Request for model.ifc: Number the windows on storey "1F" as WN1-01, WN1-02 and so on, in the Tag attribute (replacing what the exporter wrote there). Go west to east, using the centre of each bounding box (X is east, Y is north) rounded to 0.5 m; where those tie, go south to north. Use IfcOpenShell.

First a look at what the model holds.

```python
import ifcopenshell
import ifcopenshell.util.element
import ifcopenshell.util.placement

model = ifcopenshell.open("model.ifc")
print(model.schema)
storey = next(s for s in model.by_type("IfcBuildingStorey") if s.Name == "1F")
windows = [e for e in ifcopenshell.util.element.get_decomposition(storey) if e.is_a("IfcWindow")]
for e in sorted(windows, key=lambda e: e.id()):
    origin = ifcopenshell.util.placement.get_local_placement(e.ObjectPlacement)[:3, 3]
    print(e.id(), e.Tag, e.Name, origin.round(2) + 0.0, sep=" | ")
```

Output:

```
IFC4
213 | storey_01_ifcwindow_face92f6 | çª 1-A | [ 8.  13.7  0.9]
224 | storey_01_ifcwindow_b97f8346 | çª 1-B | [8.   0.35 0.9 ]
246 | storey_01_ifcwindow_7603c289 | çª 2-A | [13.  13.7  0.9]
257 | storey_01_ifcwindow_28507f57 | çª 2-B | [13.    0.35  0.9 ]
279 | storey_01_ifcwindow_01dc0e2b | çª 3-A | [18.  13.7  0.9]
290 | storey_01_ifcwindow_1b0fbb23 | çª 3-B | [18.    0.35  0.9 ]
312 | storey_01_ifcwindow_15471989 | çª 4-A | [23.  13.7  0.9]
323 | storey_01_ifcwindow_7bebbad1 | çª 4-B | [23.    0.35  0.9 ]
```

```python
import ifcopenshell
import ifcopenshell.geom
import ifcopenshell.util.element
import ifcopenshell.util.shape

model = ifcopenshell.open("model.ifc")
settings = ifcopenshell.geom.settings()
settings.set("use-world-coords", True)


def centre(element):
    shape = ifcopenshell.geom.create_shape(settings, element)
    return ifcopenshell.util.shape.get_bbox_centroid(shape.geometry)


storey = next(s for s in model.by_type("IfcBuildingStorey") if s.Name == "1F")
windows = [e for e in ifcopenshell.util.element.get_decomposition(storey) if e.is_a("IfcWindow")]

# Insertion points can sit at a corner or the storey origin, so sort by the geometry (in metres).
centres = {e: centre(e) for e in windows}
windows.sort(key=lambda e: (round(centres[e][0] / 0.5), centres[e][1]))

for i, e in enumerate(windows, start=1):
    number = f"WN1-{i:02d}"
    e.Tag = number
    print(e.id(), number)

model.write("model_edited.ifc")
```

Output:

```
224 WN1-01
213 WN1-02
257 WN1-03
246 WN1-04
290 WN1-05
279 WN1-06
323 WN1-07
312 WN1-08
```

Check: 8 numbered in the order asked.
